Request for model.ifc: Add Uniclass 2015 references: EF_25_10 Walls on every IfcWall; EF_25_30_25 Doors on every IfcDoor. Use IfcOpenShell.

First a look at what the model holds.

```python
import ifcopenshell

model = ifcopenshell.open("model.ifc")
print(model.schema)
print("classifications:", [c.Name for c in model.by_type("IfcClassification")])
for ifc_class in ("IfcDoor", "IfcRoof", "IfcStair", "IfcWall", "IfcWindow"):
    print(ifc_class, len(model.by_type(ifc_class)))
```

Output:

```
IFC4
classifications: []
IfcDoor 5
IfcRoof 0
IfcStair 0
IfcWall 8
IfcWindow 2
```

```python
import ifcopenshell
import ifcopenshell.api.classification

model = ifcopenshell.open("model.ifc")

system = ifcopenshell.api.classification.add_classification(model, classification="Uniclass 2015")

codes = {
    "IfcWall": ("EF_25_10", "Walls"),
    "IfcDoor": ("EF_25_30_25", "Doors"),
}
for ifc_class, (code, name) in codes.items():
    products = model.by_type(ifc_class)
    ifcopenshell.api.classification.add_reference(
        model, products=products, classification=system, identification=code, name=name
    )
    print(code, len(products))

model.write("model-out.ifc")
```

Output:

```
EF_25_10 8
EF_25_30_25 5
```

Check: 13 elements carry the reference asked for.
